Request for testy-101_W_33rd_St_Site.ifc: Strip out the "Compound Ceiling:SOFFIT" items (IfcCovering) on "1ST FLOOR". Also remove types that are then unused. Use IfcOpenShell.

First a look at what the model holds.

```python
import ifcopenshell
import ifcopenshell.util.element

model = ifcopenshell.open("testy-101_W_33rd_St_Site.ifc")
print(model.schema)
storey = next(s for s in model.by_type("IfcBuildingStorey") if s.Name == "1ST FLOOR")
coverings = [e for e in ifcopenshell.util.element.get_decomposition(storey) if e.is_a("IfcCovering")]
seen = {}
for e in coverings:
    element_type = ifcopenshell.util.element.get_type(e)
    name = element_type.Name if element_type not in (None, e) else None
    seen[name] = seen.get(name, 0) + 1
for name, count in sorted(seen.items(), key=str):
    print(count, "x", name)
```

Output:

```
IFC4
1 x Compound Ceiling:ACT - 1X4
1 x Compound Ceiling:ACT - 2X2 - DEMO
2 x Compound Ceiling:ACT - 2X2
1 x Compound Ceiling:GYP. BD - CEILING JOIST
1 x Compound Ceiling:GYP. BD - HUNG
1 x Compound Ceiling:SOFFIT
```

```python
import ifcopenshell
import ifcopenshell.api.root
import ifcopenshell.util.element

model = ifcopenshell.open("testy-101_W_33rd_St_Site.ifc")

storey = next(s for s in model.by_type("IfcBuildingStorey") if s.Name == "1ST FLOOR")
coverings = [e for e in ifcopenshell.util.element.get_decomposition(storey) if e.is_a("IfcCovering")]
targets = [e for e in coverings if (t := ifcopenshell.util.element.get_type(e)) not in (None, e) and t.Name == "Compound Ceiling:SOFFIT"]
types = {ifcopenshell.util.element.get_type(e) for e in targets} - {None, *targets}

for e in targets:
    ifcopenshell.api.root.remove_product(model, product=e)
print(len(targets), "removed")

unused = [t for t in types if not ifcopenshell.util.element.get_types(t)]
for t in unused:
    ifcopenshell.api.root.remove_product(model, product=t)
print(len(unused), "unused types removed")

model.write("testy-101_W_33rd_St_Site_v2.ifc")
```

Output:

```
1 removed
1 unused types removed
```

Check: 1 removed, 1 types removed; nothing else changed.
